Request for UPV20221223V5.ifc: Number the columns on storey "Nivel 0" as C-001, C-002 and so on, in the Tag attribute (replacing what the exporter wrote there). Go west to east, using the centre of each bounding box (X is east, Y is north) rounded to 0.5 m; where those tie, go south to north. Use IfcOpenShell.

First a look at what the model holds.

```python
import ifcopenshell
import ifcopenshell.util.element
import ifcopenshell.util.placement

model = ifcopenshell.open("UPV20221223V5.ifc")
print(model.schema)
storey = next(s for s in model.by_type("IfcBuildingStorey") if s.Name == "Nivel 0")
columns = [e for e in ifcopenshell.util.element.get_decomposition(storey) if e.is_a("IfcColumn")]
for e in sorted(columns, key=lambda e: e.id()):
    origin = ifcopenshell.util.placement.get_local_placement(e.ObjectPlacement)[:3, 3]
    print(e.id(), e.Tag, e.Name, origin.round(2) + 0.0, sep=" | ")
```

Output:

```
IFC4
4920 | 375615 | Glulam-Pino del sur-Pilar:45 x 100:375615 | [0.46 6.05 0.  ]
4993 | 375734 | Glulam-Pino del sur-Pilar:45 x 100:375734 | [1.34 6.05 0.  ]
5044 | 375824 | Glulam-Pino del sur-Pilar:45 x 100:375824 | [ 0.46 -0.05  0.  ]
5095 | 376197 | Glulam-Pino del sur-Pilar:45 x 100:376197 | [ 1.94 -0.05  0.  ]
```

```python
import ifcopenshell
import ifcopenshell.geom
import ifcopenshell.util.element
import ifcopenshell.util.shape

model = ifcopenshell.open("UPV20221223V5.ifc")
settings = ifcopenshell.geom.settings()
settings.set("use-world-coords", True)


def centre(element):
    shape = ifcopenshell.geom.create_shape(settings, element)
    return ifcopenshell.util.shape.get_bbox_centroid(shape.geometry)


storey = next(s for s in model.by_type("IfcBuildingStorey") if s.Name == "Nivel 0")
columns = [e for e in ifcopenshell.util.element.get_decomposition(storey) if e.is_a("IfcColumn")]

# Insertion points can sit at a corner or the storey origin, so sort by the geometry (in metres).
centres = {e: centre(e) for e in columns}
columns.sort(key=lambda e: (round(centres[e][0] / 0.5), centres[e][1]))

for i, e in enumerate(columns, start=1):
    number = f"C-0{i:02d}"
    e.Tag = number
    print(e.id(), number)

model.write("UPV20221223V5_rev.ifc")
```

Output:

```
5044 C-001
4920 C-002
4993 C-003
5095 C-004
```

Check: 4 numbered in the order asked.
